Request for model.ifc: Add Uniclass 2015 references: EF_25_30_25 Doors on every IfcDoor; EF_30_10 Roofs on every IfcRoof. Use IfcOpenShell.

First a look at what the model holds.

```python
import ifcopenshell

model = ifcopenshell.open("model.ifc")
print(model.schema)
print("classifications:", [c.Name for c in model.by_type("IfcClassification")])
for ifc_class in ("IfcDoor", "IfcRoof", "IfcStair", "IfcWall", "IfcWindow"):
    print(ifc_class, len(model.by_type(ifc_class)))
```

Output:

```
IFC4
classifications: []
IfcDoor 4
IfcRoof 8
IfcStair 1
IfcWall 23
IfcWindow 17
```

```python
import ifcopenshell
import ifcopenshell.api.classification

model = ifcopenshell.open("model.ifc")

system = ifcopenshell.api.classification.add_classification(model, classification="Uniclass 2015")

codes = {
    "IfcDoor": ("EF_25_30_25", "Doors"),
    "IfcRoof": ("EF_30_10", "Roofs"),
}
for ifc_class, (code, name) in codes.items():
    products = model.by_type(ifc_class)
    ifcopenshell.api.classification.add_reference(
        model, products=products, classification=system, identification=code, name=name
    )
    print(code, len(products))

model.write("model_updated.ifc")
```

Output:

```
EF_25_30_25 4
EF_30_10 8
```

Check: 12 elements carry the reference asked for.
